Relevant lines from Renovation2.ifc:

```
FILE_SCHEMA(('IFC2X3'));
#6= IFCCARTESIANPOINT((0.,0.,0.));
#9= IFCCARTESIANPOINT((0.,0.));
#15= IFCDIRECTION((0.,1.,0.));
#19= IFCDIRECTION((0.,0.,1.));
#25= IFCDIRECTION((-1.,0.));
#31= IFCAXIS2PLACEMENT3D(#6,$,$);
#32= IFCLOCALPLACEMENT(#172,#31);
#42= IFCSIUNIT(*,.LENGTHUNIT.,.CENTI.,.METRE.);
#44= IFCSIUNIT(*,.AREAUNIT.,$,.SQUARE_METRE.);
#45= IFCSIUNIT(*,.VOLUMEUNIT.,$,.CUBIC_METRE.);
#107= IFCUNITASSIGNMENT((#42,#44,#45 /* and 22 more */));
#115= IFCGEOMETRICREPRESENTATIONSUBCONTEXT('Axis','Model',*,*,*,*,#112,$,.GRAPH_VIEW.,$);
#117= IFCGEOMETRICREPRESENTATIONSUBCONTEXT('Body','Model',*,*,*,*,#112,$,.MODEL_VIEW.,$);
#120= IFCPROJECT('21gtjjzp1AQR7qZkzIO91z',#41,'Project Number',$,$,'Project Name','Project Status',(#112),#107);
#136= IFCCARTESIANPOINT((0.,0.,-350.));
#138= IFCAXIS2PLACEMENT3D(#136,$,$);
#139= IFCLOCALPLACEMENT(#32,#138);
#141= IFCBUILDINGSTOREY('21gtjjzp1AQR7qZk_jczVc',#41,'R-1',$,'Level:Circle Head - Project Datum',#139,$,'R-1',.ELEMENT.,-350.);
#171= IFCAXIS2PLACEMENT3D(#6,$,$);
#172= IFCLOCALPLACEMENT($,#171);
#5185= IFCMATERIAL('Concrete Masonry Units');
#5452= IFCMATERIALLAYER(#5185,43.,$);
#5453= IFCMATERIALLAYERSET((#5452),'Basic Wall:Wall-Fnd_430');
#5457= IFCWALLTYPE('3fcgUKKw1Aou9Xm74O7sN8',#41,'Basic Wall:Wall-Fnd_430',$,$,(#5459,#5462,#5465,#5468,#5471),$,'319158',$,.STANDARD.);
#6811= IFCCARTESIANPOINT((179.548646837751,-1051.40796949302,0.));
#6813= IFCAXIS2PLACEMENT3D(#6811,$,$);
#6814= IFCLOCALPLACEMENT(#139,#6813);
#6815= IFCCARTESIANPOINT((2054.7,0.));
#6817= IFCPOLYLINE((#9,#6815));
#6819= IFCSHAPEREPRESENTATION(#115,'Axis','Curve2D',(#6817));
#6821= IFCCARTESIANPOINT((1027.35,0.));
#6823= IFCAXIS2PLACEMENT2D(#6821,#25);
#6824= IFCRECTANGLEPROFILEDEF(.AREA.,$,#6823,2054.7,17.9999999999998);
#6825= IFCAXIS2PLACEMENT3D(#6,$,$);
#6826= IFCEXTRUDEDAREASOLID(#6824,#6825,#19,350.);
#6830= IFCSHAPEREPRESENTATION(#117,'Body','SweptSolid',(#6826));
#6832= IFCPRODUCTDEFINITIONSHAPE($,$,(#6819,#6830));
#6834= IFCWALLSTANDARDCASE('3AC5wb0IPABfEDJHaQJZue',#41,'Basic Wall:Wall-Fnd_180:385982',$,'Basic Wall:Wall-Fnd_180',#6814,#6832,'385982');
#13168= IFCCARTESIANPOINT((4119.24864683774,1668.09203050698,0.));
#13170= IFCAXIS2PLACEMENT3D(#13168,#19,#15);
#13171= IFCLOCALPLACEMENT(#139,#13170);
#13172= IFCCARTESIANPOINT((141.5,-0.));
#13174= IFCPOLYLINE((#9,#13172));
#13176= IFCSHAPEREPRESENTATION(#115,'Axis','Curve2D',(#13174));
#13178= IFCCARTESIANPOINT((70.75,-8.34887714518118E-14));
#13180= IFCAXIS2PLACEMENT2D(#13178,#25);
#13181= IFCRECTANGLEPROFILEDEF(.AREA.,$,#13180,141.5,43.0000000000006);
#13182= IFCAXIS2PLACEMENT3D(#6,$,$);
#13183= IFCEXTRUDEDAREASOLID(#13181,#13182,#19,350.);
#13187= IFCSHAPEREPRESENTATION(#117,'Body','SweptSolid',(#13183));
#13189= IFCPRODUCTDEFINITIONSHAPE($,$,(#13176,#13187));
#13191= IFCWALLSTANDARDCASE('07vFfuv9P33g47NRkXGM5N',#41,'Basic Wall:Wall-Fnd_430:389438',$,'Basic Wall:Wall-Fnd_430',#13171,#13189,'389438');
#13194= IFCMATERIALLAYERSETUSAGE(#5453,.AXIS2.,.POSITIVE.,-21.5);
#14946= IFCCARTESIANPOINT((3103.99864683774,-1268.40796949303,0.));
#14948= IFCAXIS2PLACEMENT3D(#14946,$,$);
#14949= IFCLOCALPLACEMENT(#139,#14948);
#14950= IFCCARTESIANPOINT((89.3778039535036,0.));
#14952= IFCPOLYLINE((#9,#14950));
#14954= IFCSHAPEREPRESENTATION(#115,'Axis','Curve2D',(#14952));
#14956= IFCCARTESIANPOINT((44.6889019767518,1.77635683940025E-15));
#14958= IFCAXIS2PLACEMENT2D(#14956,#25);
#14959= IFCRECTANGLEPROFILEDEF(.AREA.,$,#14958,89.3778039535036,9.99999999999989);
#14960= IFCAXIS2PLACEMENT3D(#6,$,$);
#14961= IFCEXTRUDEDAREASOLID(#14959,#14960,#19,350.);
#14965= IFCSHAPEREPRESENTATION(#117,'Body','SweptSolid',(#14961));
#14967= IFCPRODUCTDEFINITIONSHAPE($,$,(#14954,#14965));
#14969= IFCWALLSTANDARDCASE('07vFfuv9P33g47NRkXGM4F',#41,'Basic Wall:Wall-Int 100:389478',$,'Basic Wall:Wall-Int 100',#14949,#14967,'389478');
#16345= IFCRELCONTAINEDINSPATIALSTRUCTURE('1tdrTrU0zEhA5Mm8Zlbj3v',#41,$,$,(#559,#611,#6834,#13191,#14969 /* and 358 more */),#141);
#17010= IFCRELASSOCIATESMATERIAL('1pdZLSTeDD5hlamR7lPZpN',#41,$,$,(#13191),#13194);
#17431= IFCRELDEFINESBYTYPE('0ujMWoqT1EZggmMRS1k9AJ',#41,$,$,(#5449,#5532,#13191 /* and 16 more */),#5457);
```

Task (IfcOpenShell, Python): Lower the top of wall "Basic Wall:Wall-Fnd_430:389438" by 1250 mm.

```python
import ifcopenshell
import ifcopenshell.geom
import ifcopenshell.util.representation
import ifcopenshell.util.shape
import ifcopenshell.util.unit

model = ifcopenshell.open("Renovation2.ifc")
unit_scale = ifcopenshell.util.unit.calculate_unit_scale(model)
settings = ifcopenshell.geom.settings()


def volume(element):
    """Net volume in cubic metres, openings subtracted."""
    shape = ifcopenshell.geom.create_shape(settings, element)
    return ifcopenshell.util.shape.get_volume(shape.geometry)


wall = model.by_id(13191)
before = volume(wall)

body = ifcopenshell.util.representation.get_representation(wall, "Model", "Body")
solid = body.Items[0]
old_height = solid.Depth
solid.Depth -= 1.25 / unit_scale
after = volume(wall)

print(f"height {old_height:g} -> {solid.Depth:g}, volume {before:.3f} -> {after:.3f} m3")

model.write("Renovation2_v2.ifc")
```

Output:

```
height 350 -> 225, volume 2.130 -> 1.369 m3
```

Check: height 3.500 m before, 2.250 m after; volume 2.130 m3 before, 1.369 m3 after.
